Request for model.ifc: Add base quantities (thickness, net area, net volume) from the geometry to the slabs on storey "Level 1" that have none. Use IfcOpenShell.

First a look at what the model holds.

```python
import ifcopenshell
import ifcopenshell.util.element
import ifcopenshell.util.unit

model = ifcopenshell.open("model.ifc")
print(model.schema)
for unit_type in ("LENGTHUNIT", "AREAUNIT", "VOLUMEUNIT"):
    print(unit_type, ifcopenshell.util.unit.calculate_unit_scale(model, unit_type))
storey = next(s for s in model.by_type("IfcBuildingStorey") if s.Name == "Level 1")
slabs = [e for e in ifcopenshell.util.element.get_decomposition(storey) if e.is_a("IfcSlab")]
for e in sorted(slabs, key=lambda e: e.id()):
    print(e.id(), e.is_a(), e.Name, list(ifcopenshell.util.element.get_psets(e, qtos_only=True)), sep=" | ")
```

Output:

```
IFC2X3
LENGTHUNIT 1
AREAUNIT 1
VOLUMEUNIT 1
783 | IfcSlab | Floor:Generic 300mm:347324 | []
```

```python
import ifcopenshell
import ifcopenshell.api.pset
import ifcopenshell.geom
import ifcopenshell.util.element
import ifcopenshell.util.shape
import ifcopenshell.util.unit

model = ifcopenshell.open("model.ifc")
unit_scale = ifcopenshell.util.unit.calculate_unit_scale(model)
area_scale = ifcopenshell.util.unit.calculate_unit_scale(model, "AREAUNIT")
volume_scale = ifcopenshell.util.unit.calculate_unit_scale(model, "VOLUMEUNIT")
settings = ifcopenshell.geom.settings()

storey = next(s for s in model.by_type("IfcBuildingStorey") if s.Name == "Level 1")
slabs = [e for e in ifcopenshell.util.element.get_decomposition(storey) if e.is_a("IfcSlab")]

for e in sorted(slabs, key=lambda e: e.id()):
    if ifcopenshell.util.element.get_psets(e, qtos_only=True, should_inherit=False):
        continue
    # Geometry comes back in metres, in the element's own axes.
    shape = ifcopenshell.geom.create_shape(settings, e)
    values = {
        "Width": ifcopenshell.util.shape.get_z(shape.geometry) / unit_scale,
        "NetArea": ifcopenshell.util.shape.get_footprint_area(shape.geometry) / area_scale,
        "NetVolume": ifcopenshell.util.shape.get_volume(shape.geometry) / volume_scale,
    }
    qto = ifcopenshell.api.pset.add_qto(model, product=e, name="BaseQuantities")
    ifcopenshell.api.pset.edit_qto(model, qto=qto, properties=values)
    print(e.id(), {k: round(v, 3) for k, v in values.items()})

model.write("model_edited.ifc")
```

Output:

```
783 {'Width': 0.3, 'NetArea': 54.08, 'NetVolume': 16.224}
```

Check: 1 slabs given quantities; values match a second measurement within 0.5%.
